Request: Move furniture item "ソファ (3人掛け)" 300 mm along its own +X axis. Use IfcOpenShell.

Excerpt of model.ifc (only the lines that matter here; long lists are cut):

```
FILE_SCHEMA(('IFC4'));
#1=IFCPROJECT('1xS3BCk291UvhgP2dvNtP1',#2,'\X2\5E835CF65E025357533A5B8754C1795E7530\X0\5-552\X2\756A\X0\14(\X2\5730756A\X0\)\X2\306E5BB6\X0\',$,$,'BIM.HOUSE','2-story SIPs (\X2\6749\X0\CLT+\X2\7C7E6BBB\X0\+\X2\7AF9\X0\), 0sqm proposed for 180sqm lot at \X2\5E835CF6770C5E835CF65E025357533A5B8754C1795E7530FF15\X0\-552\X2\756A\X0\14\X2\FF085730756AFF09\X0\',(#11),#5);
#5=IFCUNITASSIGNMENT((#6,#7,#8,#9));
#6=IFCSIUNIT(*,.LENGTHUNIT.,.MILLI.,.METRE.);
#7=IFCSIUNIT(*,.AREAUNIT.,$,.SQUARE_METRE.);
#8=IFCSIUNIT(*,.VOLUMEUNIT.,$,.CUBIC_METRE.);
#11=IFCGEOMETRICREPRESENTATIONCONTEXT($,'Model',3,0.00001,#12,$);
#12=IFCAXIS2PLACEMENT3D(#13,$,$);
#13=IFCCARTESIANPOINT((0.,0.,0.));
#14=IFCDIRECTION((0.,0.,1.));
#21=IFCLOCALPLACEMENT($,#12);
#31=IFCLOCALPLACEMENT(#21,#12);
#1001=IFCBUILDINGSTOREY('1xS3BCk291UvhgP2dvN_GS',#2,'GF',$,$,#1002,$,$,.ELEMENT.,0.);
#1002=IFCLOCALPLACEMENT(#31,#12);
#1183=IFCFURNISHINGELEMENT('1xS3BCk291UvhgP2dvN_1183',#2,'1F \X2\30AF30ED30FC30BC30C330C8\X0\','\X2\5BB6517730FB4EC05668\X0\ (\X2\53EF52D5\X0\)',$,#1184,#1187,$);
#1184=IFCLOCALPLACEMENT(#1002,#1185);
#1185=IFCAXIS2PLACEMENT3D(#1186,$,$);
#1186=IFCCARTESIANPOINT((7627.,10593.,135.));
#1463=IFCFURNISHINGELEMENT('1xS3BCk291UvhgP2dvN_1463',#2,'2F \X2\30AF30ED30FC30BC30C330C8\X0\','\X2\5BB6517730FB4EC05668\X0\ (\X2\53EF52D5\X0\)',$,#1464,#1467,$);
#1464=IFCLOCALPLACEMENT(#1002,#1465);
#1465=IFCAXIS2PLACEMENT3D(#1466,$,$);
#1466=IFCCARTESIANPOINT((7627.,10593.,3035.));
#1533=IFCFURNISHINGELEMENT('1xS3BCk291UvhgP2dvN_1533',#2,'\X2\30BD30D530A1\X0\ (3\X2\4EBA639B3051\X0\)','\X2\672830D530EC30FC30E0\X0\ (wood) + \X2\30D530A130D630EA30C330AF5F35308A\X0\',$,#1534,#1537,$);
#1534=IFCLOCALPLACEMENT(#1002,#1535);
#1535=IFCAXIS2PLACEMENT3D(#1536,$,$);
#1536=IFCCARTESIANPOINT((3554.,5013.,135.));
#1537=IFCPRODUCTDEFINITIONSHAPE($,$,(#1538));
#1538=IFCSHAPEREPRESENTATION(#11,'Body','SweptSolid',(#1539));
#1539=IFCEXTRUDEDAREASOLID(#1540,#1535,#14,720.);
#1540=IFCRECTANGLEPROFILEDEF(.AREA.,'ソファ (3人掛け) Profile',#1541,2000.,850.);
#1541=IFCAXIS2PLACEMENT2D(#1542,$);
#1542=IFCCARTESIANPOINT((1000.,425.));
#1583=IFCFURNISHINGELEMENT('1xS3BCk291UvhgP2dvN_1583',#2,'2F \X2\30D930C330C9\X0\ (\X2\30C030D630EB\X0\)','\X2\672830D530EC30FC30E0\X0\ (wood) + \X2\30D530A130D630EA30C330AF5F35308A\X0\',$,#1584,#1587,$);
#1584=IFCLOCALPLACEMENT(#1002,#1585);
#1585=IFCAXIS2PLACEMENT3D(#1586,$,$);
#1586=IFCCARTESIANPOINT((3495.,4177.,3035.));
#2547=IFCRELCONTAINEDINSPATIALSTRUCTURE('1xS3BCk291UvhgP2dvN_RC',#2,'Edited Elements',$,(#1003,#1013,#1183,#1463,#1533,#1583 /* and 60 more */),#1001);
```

```python
import ifcopenshell
import ifcopenshell.api.geometry
import ifcopenshell.util.placement
import ifcopenshell.util.unit

model = ifcopenshell.open("model.ifc")
unit_scale = ifcopenshell.util.unit.calculate_unit_scale(model)

item = model.by_id(1533)
matrix = ifcopenshell.util.placement.get_local_placement(item.ObjectPlacement)
matrix[:3, 3] += matrix[:3, 0] * 0.3 / unit_scale
ifcopenshell.api.geometry.edit_object_placement(model, product=item, matrix=matrix, is_si=False)

print(ifcopenshell.util.placement.get_local_placement(item.ObjectPlacement).round(3) + 0.0)

model.write("model_rev.ifc")
```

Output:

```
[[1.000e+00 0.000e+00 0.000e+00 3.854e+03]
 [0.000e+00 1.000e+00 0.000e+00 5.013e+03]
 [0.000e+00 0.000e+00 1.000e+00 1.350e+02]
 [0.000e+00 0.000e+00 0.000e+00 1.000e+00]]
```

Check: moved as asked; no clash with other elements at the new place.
